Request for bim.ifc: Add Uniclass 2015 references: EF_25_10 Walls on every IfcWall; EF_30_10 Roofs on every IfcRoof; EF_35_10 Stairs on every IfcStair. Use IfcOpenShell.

First a look at what the model holds.

```python
import ifcopenshell

model = ifcopenshell.open("bim.ifc")
print(model.schema)
print("classifications:", [c.Name for c in model.by_type("IfcClassification")])
for ifc_class in ("IfcDoor", "IfcRoof", "IfcStair", "IfcWall", "IfcWindow"):
    print(ifc_class, len(model.by_type(ifc_class)))
```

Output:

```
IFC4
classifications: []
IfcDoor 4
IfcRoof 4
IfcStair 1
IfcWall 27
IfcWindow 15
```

```python
import ifcopenshell
import ifcopenshell.api.classification

model = ifcopenshell.open("bim.ifc")

system = ifcopenshell.api.classification.add_classification(model, classification="Uniclass 2015")

codes = {
    "IfcWall": ("EF_25_10", "Walls"),
    "IfcRoof": ("EF_30_10", "Roofs"),
    "IfcStair": ("EF_35_10", "Stairs"),
}
for ifc_class, (code, name) in codes.items():
    products = model.by_type(ifc_class)
    ifcopenshell.api.classification.add_reference(
        model, products=products, classification=system, identification=code, name=name
    )
    print(code, len(products))

model.write("bim_rev.ifc")
```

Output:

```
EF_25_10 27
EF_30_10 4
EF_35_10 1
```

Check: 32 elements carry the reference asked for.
